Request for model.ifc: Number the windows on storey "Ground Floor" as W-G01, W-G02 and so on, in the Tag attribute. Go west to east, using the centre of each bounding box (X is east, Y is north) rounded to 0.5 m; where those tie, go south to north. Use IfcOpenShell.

First a look at what the model holds.

```python
import ifcopenshell
import ifcopenshell.util.element
import ifcopenshell.util.placement

model = ifcopenshell.open("model.ifc")
print(model.schema)
storey = next(s for s in model.by_type("IfcBuildingStorey") if s.Name == "Ground Floor")
windows = [e for e in ifcopenshell.util.element.get_decomposition(storey) if e.is_a("IfcWindow")]
for e in sorted(windows, key=lambda e: e.id()):
    origin = ifcopenshell.util.placement.get_local_placement(e.ObjectPlacement)[:3, 3]
    print(e.id(), e.Tag, e.Name, origin.round(2) + 0.0, sep=" | ")
```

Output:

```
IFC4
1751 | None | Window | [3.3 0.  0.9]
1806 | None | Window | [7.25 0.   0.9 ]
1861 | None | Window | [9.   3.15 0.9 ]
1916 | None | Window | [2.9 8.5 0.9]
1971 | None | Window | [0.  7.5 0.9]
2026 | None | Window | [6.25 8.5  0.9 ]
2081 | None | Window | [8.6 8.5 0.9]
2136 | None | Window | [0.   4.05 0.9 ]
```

```python
import ifcopenshell
import ifcopenshell.geom
import ifcopenshell.util.element
import ifcopenshell.util.shape

model = ifcopenshell.open("model.ifc")
settings = ifcopenshell.geom.settings()
settings.set("use-world-coords", True)


def centre(element):
    shape = ifcopenshell.geom.create_shape(settings, element)
    return ifcopenshell.util.shape.get_bbox_centroid(shape.geometry)


storey = next(s for s in model.by_type("IfcBuildingStorey") if s.Name == "Ground Floor")
windows = [e for e in ifcopenshell.util.element.get_decomposition(storey) if e.is_a("IfcWindow")]

# Insertion points can sit at a corner or the storey origin, so sort by the geometry (in metres).
centres = {e: centre(e) for e in windows}
windows.sort(key=lambda e: (round(centres[e][0] / 0.5), centres[e][1]))

for i, e in enumerate(windows, start=1):
    number = f"W-G{i:02d}"
    e.Tag = number
    print(e.id(), number)

model.write("model_updated.ifc")
```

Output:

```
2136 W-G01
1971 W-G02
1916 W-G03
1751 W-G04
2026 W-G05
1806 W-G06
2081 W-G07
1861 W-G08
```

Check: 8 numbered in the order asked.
